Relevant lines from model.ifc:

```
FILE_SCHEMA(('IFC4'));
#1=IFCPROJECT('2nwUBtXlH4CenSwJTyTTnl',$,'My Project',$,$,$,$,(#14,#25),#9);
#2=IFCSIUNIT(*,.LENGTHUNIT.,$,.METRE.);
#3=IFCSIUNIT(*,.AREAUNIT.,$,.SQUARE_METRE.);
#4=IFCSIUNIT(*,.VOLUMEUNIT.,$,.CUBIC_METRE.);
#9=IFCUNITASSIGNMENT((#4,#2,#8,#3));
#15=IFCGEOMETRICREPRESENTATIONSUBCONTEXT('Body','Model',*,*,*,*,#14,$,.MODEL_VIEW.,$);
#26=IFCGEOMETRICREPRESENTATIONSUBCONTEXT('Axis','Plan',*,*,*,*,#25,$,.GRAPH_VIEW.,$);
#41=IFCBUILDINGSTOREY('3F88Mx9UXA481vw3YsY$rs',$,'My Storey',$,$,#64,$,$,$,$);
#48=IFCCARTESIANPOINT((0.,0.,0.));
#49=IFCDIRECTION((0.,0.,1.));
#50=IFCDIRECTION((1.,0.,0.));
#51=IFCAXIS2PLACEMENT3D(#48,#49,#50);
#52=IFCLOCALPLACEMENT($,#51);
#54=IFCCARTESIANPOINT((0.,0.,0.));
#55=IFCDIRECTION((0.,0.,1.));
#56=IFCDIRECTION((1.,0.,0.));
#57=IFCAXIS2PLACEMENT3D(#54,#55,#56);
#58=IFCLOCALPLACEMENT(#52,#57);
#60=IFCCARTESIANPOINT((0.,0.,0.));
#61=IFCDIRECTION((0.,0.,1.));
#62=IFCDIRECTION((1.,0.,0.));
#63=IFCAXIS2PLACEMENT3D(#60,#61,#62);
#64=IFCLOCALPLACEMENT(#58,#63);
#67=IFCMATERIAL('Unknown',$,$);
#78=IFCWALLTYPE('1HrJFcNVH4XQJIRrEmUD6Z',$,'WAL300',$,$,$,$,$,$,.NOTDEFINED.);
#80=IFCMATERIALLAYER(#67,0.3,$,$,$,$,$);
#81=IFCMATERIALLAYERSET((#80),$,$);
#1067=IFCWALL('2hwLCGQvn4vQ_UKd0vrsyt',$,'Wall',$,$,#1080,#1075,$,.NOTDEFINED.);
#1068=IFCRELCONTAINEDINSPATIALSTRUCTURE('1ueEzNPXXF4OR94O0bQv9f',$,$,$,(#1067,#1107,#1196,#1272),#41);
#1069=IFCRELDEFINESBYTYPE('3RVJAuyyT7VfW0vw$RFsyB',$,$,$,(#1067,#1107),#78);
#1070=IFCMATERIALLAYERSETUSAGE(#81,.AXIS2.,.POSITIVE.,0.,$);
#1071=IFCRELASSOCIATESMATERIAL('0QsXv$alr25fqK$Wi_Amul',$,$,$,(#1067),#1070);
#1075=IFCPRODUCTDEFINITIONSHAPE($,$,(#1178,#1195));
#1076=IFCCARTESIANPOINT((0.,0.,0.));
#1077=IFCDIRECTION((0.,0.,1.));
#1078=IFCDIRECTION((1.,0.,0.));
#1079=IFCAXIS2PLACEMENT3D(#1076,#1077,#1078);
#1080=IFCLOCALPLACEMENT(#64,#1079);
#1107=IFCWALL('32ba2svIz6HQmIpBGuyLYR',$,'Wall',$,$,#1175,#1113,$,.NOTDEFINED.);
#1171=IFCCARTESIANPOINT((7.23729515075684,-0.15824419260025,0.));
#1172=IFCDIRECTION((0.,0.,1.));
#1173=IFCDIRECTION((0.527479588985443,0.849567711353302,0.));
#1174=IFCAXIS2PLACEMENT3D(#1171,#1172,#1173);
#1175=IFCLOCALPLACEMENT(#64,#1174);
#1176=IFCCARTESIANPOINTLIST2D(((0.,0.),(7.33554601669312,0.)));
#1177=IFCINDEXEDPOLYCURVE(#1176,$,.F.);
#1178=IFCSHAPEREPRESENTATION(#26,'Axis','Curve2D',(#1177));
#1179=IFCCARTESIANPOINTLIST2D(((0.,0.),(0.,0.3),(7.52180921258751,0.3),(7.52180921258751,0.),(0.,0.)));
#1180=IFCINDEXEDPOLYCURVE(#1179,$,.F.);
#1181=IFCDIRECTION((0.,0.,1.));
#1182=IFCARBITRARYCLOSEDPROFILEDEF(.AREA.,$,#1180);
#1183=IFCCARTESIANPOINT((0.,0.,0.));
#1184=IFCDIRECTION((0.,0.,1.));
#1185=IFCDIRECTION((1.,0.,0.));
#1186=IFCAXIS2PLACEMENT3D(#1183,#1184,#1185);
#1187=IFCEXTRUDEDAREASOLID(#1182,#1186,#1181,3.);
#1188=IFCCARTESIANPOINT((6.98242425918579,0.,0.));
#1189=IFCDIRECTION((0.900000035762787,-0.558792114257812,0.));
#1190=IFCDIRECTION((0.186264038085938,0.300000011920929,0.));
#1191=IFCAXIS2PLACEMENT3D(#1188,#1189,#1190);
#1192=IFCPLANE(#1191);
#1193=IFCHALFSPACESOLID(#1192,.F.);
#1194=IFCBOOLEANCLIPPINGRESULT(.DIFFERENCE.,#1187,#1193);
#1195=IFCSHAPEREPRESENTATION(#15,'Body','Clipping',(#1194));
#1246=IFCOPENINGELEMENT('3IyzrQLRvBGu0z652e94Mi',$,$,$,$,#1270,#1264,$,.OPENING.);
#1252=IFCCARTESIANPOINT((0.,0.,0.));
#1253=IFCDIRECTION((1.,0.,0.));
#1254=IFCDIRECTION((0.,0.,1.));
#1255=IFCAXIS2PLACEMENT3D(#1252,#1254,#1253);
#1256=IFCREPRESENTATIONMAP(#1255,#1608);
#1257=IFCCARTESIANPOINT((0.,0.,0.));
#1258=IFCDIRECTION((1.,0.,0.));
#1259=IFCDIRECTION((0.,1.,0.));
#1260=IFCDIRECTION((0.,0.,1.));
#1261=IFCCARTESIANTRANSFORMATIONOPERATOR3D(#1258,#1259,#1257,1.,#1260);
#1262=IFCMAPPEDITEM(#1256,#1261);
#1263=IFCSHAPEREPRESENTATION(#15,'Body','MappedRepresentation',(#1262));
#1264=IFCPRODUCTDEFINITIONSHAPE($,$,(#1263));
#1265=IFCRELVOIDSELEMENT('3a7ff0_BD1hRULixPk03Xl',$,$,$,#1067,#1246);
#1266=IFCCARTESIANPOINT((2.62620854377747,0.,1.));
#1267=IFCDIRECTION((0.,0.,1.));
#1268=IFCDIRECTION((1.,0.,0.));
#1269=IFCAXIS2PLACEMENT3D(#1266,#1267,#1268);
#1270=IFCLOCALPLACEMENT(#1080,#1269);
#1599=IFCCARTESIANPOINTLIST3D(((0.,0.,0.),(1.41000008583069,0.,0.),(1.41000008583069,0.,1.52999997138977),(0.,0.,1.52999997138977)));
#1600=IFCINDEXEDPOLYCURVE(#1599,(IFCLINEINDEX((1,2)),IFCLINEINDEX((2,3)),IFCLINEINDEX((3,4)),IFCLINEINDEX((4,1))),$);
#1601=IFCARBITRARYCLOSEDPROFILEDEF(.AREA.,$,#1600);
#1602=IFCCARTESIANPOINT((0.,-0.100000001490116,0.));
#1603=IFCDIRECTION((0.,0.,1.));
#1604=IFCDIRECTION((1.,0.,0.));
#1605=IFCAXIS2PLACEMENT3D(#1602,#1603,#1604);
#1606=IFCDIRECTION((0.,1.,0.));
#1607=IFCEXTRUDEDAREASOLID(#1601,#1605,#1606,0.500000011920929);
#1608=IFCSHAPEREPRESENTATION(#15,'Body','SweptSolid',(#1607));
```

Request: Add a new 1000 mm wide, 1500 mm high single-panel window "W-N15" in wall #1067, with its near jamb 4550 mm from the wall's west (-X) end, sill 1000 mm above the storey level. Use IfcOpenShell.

```python
import numpy as np
import ifcopenshell
import ifcopenshell.api.feature
import ifcopenshell.api.geometry
import ifcopenshell.api.root
import ifcopenshell.api.spatial
import ifcopenshell.geom
import ifcopenshell.util.element
import ifcopenshell.util.placement
import ifcopenshell.util.representation
import ifcopenshell.util.shape
import ifcopenshell.util.unit

model = ifcopenshell.open("model.ifc")
unit_scale = ifcopenshell.util.unit.calculate_unit_scale(model)
settings = ifcopenshell.geom.settings()


def volume(element):
    """Net volume in cubic metres, openings subtracted."""
    shape = ifcopenshell.geom.create_shape(settings, element)
    return ifcopenshell.util.shape.get_volume(shape.geometry)


wall = model.by_guid("2hwLCGQvn4vQ_UKd0vrsyt")
storey = ifcopenshell.util.element.get_container(wall, ifc_class="IfcBuildingStorey")
context = ifcopenshell.util.representation.get_context(model, "Model", "Body", "MODEL_VIEW")
before = volume(wall)

width, height, from_end, sill = 1, 1.5, 4.55, 1  # metres

# The wall runs along its own X axis, and the end named is its -X end.
wall_shape = ifcopenshell.geom.create_shape(settings, wall)
x, y, z = ifcopenshell.util.shape.get_vertices(wall_shape.geometry).T
start = x.min() + from_end
face, thickness = float(y.min()), float(y.max() - y.min())
wall_matrix = ifcopenshell.util.placement.get_local_placement(wall.ObjectPlacement)
level = ifcopenshell.util.placement.get_local_placement(storey.ObjectPlacement)[2, 3]


def in_wall(x, y):
    """Placement at x, y metres in the wall's axes, at sill height."""
    matrix = wall_matrix.copy()
    matrix[:, 3] = wall_matrix @ np.array([x / unit_scale, y / unit_scale, 0.0, 1.0])
    matrix[2, 3] = level + sill / unit_scale
    return matrix


# Opening: a box that overshoots both wall faces by 50 mm.
opening = ifcopenshell.api.root.create_entity(model, ifc_class="IfcOpeningElement", predefined_type="OPENING")
box = ifcopenshell.api.geometry.add_wall_representation(
    model, context=context, length=width, height=height, thickness=thickness + 0.1
)
ifcopenshell.api.geometry.assign_representation(model, product=opening, representation=box)
ifcopenshell.api.geometry.edit_object_placement(model, product=opening, matrix=in_wall(start, face - 0.05), is_si=False)
ifcopenshell.api.feature.add_feature(model, feature=opening, element=wall)

window = ifcopenshell.api.root.create_entity(model, ifc_class="IfcWindow", name="W-N15", predefined_type="WINDOW")
window.OverallWidth, window.OverallHeight = width / unit_scale, height / unit_scale
window.PartitioningType = "SINGLE_PANEL"
body = ifcopenshell.api.geometry.add_window_representation(
    model,
    context=context,
    overall_width=window.OverallWidth,
    overall_height=window.OverallHeight,
    partition_type="SINGLE_PANEL",
)
ifcopenshell.api.geometry.assign_representation(model, product=window, representation=body)
ifcopenshell.api.spatial.assign_container(model, products=[window], relating_structure=storey)
ifcopenshell.api.feature.add_filling(model, opening=opening, element=window)

# Centre the window in the wall's thickness.
ifcopenshell.api.geometry.edit_object_placement(model, product=window, matrix=in_wall(start, face), is_si=False)
window_shape = ifcopenshell.geom.create_shape(settings, window)
depth = ifcopenshell.util.shape.get_vertices(window_shape.geometry)[:, 1]
offset = face + thickness / 2 - (depth.min() + depth.max()) / 2
ifcopenshell.api.geometry.edit_object_placement(model, product=window, matrix=in_wall(start, offset), is_si=False)

after = volume(wall)

print(f"wall volume {before:.3f} -> {after:.3f} m3")

model.write("model_rev.ifc")
```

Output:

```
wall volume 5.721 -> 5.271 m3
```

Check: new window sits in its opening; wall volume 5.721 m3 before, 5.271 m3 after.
